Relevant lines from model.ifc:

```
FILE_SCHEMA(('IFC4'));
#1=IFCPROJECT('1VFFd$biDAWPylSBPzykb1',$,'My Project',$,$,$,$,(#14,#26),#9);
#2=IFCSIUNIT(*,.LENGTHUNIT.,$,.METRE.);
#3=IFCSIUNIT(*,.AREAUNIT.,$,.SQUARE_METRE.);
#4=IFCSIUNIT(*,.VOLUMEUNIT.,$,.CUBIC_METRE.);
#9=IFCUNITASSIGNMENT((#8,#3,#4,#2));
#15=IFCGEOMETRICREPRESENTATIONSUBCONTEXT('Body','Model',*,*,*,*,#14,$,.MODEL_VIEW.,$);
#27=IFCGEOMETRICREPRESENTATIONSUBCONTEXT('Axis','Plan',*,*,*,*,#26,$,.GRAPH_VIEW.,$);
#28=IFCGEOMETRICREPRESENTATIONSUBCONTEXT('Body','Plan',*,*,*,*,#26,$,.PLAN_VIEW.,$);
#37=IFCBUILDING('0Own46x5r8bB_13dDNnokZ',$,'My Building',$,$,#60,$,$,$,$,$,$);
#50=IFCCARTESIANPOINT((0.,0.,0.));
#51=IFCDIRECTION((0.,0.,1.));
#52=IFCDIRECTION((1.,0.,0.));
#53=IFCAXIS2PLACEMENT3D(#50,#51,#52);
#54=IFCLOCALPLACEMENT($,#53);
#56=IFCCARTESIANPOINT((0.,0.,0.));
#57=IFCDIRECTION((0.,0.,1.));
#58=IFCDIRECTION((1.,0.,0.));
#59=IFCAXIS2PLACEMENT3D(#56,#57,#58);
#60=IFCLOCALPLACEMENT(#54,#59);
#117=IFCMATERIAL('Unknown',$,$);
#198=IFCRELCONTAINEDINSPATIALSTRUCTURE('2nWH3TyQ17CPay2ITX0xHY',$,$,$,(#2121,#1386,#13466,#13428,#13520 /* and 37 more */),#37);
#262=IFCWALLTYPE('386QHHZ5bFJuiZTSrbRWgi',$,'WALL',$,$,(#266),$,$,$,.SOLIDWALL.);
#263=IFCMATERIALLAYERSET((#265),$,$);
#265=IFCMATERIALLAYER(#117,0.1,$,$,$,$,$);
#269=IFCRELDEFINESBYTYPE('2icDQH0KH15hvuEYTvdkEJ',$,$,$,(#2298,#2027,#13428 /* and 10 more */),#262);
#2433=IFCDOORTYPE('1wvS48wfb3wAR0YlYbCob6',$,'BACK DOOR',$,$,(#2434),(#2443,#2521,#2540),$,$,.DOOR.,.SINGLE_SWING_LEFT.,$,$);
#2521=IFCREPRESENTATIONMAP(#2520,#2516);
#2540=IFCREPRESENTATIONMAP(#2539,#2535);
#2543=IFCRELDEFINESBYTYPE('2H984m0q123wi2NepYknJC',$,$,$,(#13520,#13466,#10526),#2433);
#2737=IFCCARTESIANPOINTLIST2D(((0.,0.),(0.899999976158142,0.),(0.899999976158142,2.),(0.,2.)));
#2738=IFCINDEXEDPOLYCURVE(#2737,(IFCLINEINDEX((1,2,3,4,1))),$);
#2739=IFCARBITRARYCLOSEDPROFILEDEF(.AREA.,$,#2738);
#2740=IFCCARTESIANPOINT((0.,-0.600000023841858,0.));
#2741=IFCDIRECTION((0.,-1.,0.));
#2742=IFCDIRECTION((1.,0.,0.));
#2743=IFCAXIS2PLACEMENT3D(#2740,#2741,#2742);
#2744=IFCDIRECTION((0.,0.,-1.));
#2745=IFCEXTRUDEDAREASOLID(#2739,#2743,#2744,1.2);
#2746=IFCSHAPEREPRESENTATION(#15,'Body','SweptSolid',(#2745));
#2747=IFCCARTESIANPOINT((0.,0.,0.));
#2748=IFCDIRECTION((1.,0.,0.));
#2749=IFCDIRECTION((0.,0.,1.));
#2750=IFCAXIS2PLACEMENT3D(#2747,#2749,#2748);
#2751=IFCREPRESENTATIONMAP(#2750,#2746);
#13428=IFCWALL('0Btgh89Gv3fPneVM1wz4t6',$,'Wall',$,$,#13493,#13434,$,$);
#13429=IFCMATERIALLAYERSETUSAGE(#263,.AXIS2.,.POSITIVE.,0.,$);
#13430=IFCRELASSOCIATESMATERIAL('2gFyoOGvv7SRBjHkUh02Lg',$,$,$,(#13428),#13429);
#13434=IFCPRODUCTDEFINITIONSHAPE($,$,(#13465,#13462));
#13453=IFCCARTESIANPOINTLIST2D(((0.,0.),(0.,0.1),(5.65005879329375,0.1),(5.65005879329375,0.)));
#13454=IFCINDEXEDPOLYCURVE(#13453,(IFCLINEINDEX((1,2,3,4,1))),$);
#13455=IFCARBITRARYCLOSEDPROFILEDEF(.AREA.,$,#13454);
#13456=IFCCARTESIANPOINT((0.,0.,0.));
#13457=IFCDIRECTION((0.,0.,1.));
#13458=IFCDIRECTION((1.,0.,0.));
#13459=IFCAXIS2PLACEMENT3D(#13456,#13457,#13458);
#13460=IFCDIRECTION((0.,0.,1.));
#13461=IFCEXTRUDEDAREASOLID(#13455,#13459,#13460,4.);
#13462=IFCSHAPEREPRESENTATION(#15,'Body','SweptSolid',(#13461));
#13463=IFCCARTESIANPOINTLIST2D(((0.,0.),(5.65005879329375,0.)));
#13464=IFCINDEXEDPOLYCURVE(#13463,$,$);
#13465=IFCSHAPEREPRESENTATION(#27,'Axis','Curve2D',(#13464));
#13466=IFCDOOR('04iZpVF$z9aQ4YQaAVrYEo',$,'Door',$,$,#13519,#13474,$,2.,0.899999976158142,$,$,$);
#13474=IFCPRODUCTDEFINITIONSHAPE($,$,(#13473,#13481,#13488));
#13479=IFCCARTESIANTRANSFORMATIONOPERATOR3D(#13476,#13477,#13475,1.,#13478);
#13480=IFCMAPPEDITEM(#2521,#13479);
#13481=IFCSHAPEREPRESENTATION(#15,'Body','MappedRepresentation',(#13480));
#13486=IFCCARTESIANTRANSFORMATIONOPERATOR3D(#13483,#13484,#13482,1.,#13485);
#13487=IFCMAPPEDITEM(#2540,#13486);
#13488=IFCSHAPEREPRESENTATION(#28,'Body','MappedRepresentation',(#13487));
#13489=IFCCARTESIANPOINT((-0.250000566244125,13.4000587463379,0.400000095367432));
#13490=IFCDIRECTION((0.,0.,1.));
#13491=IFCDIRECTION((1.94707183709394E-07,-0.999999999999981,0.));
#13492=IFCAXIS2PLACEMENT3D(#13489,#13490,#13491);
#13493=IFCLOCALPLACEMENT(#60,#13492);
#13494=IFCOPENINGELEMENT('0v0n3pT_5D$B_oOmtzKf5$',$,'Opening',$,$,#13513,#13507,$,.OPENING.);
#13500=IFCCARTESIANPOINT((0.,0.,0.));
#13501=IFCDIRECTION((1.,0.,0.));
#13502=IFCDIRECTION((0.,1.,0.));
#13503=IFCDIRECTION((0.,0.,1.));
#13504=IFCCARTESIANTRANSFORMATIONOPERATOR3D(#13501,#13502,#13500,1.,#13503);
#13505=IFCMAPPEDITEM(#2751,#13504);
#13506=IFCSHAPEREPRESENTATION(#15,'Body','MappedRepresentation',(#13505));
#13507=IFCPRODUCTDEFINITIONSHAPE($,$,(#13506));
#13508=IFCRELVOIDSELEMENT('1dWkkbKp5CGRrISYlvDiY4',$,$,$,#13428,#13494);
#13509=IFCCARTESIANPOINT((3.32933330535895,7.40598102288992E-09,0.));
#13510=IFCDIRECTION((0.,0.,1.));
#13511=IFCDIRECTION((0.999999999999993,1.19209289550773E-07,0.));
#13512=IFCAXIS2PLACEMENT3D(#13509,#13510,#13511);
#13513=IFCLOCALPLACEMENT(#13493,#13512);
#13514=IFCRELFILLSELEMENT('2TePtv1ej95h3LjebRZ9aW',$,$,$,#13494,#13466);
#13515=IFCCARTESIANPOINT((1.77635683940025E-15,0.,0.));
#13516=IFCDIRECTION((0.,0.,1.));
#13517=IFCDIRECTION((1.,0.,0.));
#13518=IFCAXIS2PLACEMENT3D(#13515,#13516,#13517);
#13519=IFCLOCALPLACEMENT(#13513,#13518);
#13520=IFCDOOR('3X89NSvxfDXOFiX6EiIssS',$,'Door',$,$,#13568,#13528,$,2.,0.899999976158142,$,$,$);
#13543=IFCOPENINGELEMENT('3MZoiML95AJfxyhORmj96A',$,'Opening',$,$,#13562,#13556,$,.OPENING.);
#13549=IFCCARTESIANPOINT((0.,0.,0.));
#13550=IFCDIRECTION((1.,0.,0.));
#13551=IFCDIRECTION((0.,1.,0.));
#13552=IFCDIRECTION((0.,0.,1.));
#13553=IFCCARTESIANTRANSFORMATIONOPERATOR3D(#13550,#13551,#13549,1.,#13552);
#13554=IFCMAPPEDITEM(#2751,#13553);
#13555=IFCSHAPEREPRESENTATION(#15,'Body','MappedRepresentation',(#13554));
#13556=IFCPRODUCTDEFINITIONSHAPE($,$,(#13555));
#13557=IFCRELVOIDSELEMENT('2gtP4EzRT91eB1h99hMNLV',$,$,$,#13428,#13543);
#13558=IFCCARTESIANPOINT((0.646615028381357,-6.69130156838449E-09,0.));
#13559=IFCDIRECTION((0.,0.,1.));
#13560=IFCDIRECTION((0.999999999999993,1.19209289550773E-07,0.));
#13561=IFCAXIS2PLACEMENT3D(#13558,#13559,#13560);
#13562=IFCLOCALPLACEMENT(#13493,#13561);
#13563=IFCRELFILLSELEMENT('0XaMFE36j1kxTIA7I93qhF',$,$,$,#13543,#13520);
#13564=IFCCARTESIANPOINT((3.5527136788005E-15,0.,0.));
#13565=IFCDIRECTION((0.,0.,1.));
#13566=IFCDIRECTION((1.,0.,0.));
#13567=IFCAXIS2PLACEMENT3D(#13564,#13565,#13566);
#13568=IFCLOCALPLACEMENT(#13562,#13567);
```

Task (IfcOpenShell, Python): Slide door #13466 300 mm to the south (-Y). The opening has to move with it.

```python
import ifcopenshell
import ifcopenshell.api.geometry
import ifcopenshell.util.placement

model = ifcopenshell.open("model.ifc")

door = model.by_guid("04iZpVF$z9aQ4YQaAVrYEo")
opening = door.FillsVoids[0].RelatingOpeningElement
wall = opening.VoidsElements[0].RelatingBuildingElement

wall_matrix = ifcopenshell.util.placement.get_local_placement(wall.ObjectPlacement)
shift = wall_matrix[:3, 0] * 0.3
before = ifcopenshell.util.placement.get_local_placement(door.ObjectPlacement)[:3, 3].copy()

# The door is placed relative to its opening, so it follows when the opening moves.
matrix = ifcopenshell.util.placement.get_local_placement(opening.ObjectPlacement)
matrix[:3, 3] += shift
ifcopenshell.api.geometry.edit_object_placement(
    model, product=opening, matrix=matrix, is_si=False, should_transform_children=True
)

after = ifcopenshell.util.placement.get_local_placement(door.ObjectPlacement)[:3, 3]
print("door moved by", (after - before).round(3) + 0.0)

model.write("model_edited.ifc")
```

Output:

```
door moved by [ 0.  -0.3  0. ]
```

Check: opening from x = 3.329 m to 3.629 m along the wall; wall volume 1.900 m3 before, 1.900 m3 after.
